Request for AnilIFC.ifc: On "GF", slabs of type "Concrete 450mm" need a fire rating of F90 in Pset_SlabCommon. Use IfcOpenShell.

First a look at what the model holds.

```python
import ifcopenshell
import ifcopenshell.util.element

model = ifcopenshell.open("AnilIFC.ifc")
print(model.schema)
storey = next(s for s in model.by_type("IfcBuildingStorey") if s.Name == "GF")
slabs = [e for e in ifcopenshell.util.element.get_decomposition(storey) if e.is_a("IfcSlab")]
seen = {}
for e in slabs:
    element_type = ifcopenshell.util.element.get_type(e)
    key = (element_type.Name if element_type != e and element_type else None, ifcopenshell.util.element.get_pset(e, "Pset_SlabCommon", "FireRating"))
    seen[key] = seen.get(key, 0) + 1
for (name, value), count in sorted(seen.items(), key=str):
    print(count, "x", name, "|", value)
```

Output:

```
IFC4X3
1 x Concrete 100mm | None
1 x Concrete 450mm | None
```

```python
import ifcopenshell
import ifcopenshell.api.pset
import ifcopenshell.util.element

model = ifcopenshell.open("AnilIFC.ifc")

storey = next(s for s in model.by_type("IfcBuildingStorey") if s.Name == "GF")
slabs = [e for e in ifcopenshell.util.element.get_decomposition(storey) if e.is_a("IfcSlab")]

count = 0
for e in slabs:
    element_type = ifcopenshell.util.element.get_type(e)
    if element_type in (None, e) or element_type.Name != "Concrete 450mm":
        continue
    # add_pset returns the element's existing set when there is one.
    pset = ifcopenshell.api.pset.add_pset(model, product=e, name="Pset_SlabCommon")
    ifcopenshell.api.pset.edit_pset(model, pset=pset, properties={"FireRating": "F90"})
    count += 1

print(count, "slabs updated")

model.write("AnilIFC_updated.ifc")
```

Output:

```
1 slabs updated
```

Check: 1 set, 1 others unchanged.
